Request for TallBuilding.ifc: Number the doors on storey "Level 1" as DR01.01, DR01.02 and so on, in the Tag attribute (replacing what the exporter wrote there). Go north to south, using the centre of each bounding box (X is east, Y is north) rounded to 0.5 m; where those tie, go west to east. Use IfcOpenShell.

First a look at what the model holds.

```python
import ifcopenshell
import ifcopenshell.util.element
import ifcopenshell.util.placement

model = ifcopenshell.open("TallBuilding.ifc")
print(model.schema)
storey = next(s for s in model.by_type("IfcBuildingStorey") if s.Name == "Level 1")
doors = [e for e in ifcopenshell.util.element.get_decomposition(storey) if e.is_a("IfcDoor")]
for e in sorted(doors, key=lambda e: e.id()):
    origin = ifcopenshell.util.placement.get_local_placement(e.ObjectPlacement)[:3, 3]
    print(e.id(), e.Tag, e.Name, origin.round(2) + 0.0, sep=" | ")
```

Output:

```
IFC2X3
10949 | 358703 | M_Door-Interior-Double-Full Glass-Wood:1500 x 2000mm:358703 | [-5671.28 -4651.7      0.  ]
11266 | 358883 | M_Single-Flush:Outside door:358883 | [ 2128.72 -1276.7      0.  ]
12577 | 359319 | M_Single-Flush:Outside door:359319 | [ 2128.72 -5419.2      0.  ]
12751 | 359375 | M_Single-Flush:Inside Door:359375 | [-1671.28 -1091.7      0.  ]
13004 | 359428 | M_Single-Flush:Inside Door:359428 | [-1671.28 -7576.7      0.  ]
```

```python
import ifcopenshell
import ifcopenshell.geom
import ifcopenshell.util.element
import ifcopenshell.util.shape

model = ifcopenshell.open("TallBuilding.ifc")
settings = ifcopenshell.geom.settings()
settings.set("use-world-coords", True)


def centre(element):
    shape = ifcopenshell.geom.create_shape(settings, element)
    return ifcopenshell.util.shape.get_bbox_centroid(shape.geometry)


storey = next(s for s in model.by_type("IfcBuildingStorey") if s.Name == "Level 1")
doors = [e for e in ifcopenshell.util.element.get_decomposition(storey) if e.is_a("IfcDoor")]

# Insertion points can sit at a corner or the storey origin, so sort by the geometry (in metres).
centres = {e: centre(e) for e in doors}
doors.sort(key=lambda e: (-round(centres[e][1] / 0.5), centres[e][0]))

for i, e in enumerate(doors, start=1):
    number = f"DR01.{i:02d}"
    e.Tag = number
    print(e.id(), number)

model.write("TallBuilding_updated.ifc")
```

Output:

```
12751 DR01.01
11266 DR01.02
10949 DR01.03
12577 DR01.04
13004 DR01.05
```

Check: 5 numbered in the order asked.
